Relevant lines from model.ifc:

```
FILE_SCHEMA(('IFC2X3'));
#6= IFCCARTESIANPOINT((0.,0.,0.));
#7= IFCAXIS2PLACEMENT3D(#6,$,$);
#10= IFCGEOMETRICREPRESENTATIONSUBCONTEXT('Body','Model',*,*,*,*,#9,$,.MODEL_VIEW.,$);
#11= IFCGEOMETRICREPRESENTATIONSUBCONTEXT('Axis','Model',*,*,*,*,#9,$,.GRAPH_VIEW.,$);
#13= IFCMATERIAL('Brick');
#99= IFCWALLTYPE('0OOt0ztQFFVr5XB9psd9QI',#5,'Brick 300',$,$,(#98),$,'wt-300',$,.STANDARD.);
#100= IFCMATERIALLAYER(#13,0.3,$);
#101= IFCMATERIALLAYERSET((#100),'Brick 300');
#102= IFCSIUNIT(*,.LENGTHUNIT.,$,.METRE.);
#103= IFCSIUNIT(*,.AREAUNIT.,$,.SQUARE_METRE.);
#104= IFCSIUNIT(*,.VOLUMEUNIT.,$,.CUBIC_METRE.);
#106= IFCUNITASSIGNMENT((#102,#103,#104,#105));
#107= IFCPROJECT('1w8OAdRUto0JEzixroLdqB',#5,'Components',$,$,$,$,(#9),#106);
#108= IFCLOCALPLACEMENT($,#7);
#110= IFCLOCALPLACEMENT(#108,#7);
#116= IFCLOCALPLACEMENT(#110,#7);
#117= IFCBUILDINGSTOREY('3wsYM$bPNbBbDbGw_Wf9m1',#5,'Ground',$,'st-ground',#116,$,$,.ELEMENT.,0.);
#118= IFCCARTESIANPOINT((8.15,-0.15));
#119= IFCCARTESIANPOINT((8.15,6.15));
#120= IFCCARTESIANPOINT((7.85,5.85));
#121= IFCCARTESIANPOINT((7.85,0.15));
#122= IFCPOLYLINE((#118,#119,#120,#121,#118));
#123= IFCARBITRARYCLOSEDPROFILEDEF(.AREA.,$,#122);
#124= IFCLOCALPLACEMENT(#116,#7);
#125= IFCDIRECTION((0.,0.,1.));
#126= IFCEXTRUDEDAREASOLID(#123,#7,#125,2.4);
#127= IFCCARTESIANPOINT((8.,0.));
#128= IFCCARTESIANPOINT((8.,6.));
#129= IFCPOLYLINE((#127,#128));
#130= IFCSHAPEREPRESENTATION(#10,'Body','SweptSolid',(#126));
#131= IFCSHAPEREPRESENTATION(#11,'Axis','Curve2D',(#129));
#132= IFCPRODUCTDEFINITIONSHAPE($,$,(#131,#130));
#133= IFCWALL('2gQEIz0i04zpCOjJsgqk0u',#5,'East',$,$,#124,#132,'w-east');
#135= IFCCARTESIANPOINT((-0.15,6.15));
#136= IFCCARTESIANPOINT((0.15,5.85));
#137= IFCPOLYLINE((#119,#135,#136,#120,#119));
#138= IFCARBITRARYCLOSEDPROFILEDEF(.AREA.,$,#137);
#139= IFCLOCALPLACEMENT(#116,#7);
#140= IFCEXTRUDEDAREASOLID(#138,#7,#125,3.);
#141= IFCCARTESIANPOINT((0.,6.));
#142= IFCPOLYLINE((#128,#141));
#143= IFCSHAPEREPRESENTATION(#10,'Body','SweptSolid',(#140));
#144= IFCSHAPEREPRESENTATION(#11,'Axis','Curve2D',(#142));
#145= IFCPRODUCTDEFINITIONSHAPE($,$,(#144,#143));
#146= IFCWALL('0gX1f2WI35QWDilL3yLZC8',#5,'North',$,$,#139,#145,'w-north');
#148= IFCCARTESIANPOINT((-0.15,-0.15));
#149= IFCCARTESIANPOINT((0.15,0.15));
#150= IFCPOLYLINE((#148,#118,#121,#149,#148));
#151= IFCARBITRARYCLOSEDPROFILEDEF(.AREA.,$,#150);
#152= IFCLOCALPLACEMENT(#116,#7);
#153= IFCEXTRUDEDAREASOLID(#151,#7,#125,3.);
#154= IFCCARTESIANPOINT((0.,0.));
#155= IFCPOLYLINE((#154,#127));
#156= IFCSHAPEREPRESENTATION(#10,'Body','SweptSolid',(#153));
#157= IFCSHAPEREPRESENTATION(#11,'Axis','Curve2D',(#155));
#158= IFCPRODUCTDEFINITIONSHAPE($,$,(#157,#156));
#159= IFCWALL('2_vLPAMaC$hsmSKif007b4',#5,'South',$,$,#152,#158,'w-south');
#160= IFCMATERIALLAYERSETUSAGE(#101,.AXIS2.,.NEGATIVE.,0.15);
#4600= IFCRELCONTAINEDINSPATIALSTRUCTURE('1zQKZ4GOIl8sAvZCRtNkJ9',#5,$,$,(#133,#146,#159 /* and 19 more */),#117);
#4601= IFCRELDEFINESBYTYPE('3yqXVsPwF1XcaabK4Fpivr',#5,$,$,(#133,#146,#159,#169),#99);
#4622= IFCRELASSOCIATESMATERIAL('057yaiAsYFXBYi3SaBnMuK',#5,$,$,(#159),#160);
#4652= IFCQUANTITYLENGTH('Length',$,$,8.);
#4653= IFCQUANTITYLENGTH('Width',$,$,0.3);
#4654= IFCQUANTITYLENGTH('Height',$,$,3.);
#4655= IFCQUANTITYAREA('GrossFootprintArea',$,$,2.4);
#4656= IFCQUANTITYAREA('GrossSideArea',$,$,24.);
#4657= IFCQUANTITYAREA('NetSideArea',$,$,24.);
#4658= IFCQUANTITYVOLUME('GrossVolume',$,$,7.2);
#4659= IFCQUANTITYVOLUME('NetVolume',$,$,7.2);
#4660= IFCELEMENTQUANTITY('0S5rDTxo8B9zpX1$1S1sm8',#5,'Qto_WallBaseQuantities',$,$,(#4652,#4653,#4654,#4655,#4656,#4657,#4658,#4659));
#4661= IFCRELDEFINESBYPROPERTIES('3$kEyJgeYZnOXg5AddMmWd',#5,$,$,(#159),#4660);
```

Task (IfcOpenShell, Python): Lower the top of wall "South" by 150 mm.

```python
import ifcopenshell
import ifcopenshell.api.pset
import ifcopenshell.geom
import ifcopenshell.util.element
import ifcopenshell.util.representation
import ifcopenshell.util.shape
import ifcopenshell.util.unit

model = ifcopenshell.open("model.ifc")
unit_scale = ifcopenshell.util.unit.calculate_unit_scale(model)
area_scale = ifcopenshell.util.unit.calculate_unit_scale(model, "AREAUNIT")
volume_scale = ifcopenshell.util.unit.calculate_unit_scale(model, "VOLUMEUNIT")
settings = ifcopenshell.geom.settings()


def volume(element):
    """Net volume in cubic metres, openings subtracted."""
    shape = ifcopenshell.geom.create_shape(settings, element)
    return ifcopenshell.util.shape.get_volume(shape.geometry)


wall = model.by_guid("2_vLPAMaC$hsmSKif007b4")
before = volume(wall)

body = ifcopenshell.util.representation.get_representation(wall, "Model", "Body")
solid = body.Items[0]
old_height = solid.Depth
solid.Depth -= 0.15 / unit_scale
after = volume(wall)
thickness = 0.3  # wall thickness in metres

# Update the stored height, areas and volumes.
qto = model.by_id(ifcopenshell.util.element.get_pset(wall, "Qto_WallBaseQuantities", should_inherit=False)["id"])
ifcopenshell.api.pset.edit_qto(model, qto=qto, properties={
    "Height": solid.Depth,
    "GrossSideArea": ifcopenshell.util.element.get_pset(wall, "Qto_WallBaseQuantities", "GrossSideArea") * solid.Depth / old_height,
    "NetSideArea": after / thickness / area_scale,
    "GrossVolume": ifcopenshell.util.element.get_pset(wall, "Qto_WallBaseQuantities", "GrossVolume") * solid.Depth / old_height,
    "NetVolume": after / volume_scale,
})

print(f"height {old_height:g} -> {solid.Depth:g}, volume {before:.3f} -> {after:.3f} m3")

model.write("model_updated.ifc")
```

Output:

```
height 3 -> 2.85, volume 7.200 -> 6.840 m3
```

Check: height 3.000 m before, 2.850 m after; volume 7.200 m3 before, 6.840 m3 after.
